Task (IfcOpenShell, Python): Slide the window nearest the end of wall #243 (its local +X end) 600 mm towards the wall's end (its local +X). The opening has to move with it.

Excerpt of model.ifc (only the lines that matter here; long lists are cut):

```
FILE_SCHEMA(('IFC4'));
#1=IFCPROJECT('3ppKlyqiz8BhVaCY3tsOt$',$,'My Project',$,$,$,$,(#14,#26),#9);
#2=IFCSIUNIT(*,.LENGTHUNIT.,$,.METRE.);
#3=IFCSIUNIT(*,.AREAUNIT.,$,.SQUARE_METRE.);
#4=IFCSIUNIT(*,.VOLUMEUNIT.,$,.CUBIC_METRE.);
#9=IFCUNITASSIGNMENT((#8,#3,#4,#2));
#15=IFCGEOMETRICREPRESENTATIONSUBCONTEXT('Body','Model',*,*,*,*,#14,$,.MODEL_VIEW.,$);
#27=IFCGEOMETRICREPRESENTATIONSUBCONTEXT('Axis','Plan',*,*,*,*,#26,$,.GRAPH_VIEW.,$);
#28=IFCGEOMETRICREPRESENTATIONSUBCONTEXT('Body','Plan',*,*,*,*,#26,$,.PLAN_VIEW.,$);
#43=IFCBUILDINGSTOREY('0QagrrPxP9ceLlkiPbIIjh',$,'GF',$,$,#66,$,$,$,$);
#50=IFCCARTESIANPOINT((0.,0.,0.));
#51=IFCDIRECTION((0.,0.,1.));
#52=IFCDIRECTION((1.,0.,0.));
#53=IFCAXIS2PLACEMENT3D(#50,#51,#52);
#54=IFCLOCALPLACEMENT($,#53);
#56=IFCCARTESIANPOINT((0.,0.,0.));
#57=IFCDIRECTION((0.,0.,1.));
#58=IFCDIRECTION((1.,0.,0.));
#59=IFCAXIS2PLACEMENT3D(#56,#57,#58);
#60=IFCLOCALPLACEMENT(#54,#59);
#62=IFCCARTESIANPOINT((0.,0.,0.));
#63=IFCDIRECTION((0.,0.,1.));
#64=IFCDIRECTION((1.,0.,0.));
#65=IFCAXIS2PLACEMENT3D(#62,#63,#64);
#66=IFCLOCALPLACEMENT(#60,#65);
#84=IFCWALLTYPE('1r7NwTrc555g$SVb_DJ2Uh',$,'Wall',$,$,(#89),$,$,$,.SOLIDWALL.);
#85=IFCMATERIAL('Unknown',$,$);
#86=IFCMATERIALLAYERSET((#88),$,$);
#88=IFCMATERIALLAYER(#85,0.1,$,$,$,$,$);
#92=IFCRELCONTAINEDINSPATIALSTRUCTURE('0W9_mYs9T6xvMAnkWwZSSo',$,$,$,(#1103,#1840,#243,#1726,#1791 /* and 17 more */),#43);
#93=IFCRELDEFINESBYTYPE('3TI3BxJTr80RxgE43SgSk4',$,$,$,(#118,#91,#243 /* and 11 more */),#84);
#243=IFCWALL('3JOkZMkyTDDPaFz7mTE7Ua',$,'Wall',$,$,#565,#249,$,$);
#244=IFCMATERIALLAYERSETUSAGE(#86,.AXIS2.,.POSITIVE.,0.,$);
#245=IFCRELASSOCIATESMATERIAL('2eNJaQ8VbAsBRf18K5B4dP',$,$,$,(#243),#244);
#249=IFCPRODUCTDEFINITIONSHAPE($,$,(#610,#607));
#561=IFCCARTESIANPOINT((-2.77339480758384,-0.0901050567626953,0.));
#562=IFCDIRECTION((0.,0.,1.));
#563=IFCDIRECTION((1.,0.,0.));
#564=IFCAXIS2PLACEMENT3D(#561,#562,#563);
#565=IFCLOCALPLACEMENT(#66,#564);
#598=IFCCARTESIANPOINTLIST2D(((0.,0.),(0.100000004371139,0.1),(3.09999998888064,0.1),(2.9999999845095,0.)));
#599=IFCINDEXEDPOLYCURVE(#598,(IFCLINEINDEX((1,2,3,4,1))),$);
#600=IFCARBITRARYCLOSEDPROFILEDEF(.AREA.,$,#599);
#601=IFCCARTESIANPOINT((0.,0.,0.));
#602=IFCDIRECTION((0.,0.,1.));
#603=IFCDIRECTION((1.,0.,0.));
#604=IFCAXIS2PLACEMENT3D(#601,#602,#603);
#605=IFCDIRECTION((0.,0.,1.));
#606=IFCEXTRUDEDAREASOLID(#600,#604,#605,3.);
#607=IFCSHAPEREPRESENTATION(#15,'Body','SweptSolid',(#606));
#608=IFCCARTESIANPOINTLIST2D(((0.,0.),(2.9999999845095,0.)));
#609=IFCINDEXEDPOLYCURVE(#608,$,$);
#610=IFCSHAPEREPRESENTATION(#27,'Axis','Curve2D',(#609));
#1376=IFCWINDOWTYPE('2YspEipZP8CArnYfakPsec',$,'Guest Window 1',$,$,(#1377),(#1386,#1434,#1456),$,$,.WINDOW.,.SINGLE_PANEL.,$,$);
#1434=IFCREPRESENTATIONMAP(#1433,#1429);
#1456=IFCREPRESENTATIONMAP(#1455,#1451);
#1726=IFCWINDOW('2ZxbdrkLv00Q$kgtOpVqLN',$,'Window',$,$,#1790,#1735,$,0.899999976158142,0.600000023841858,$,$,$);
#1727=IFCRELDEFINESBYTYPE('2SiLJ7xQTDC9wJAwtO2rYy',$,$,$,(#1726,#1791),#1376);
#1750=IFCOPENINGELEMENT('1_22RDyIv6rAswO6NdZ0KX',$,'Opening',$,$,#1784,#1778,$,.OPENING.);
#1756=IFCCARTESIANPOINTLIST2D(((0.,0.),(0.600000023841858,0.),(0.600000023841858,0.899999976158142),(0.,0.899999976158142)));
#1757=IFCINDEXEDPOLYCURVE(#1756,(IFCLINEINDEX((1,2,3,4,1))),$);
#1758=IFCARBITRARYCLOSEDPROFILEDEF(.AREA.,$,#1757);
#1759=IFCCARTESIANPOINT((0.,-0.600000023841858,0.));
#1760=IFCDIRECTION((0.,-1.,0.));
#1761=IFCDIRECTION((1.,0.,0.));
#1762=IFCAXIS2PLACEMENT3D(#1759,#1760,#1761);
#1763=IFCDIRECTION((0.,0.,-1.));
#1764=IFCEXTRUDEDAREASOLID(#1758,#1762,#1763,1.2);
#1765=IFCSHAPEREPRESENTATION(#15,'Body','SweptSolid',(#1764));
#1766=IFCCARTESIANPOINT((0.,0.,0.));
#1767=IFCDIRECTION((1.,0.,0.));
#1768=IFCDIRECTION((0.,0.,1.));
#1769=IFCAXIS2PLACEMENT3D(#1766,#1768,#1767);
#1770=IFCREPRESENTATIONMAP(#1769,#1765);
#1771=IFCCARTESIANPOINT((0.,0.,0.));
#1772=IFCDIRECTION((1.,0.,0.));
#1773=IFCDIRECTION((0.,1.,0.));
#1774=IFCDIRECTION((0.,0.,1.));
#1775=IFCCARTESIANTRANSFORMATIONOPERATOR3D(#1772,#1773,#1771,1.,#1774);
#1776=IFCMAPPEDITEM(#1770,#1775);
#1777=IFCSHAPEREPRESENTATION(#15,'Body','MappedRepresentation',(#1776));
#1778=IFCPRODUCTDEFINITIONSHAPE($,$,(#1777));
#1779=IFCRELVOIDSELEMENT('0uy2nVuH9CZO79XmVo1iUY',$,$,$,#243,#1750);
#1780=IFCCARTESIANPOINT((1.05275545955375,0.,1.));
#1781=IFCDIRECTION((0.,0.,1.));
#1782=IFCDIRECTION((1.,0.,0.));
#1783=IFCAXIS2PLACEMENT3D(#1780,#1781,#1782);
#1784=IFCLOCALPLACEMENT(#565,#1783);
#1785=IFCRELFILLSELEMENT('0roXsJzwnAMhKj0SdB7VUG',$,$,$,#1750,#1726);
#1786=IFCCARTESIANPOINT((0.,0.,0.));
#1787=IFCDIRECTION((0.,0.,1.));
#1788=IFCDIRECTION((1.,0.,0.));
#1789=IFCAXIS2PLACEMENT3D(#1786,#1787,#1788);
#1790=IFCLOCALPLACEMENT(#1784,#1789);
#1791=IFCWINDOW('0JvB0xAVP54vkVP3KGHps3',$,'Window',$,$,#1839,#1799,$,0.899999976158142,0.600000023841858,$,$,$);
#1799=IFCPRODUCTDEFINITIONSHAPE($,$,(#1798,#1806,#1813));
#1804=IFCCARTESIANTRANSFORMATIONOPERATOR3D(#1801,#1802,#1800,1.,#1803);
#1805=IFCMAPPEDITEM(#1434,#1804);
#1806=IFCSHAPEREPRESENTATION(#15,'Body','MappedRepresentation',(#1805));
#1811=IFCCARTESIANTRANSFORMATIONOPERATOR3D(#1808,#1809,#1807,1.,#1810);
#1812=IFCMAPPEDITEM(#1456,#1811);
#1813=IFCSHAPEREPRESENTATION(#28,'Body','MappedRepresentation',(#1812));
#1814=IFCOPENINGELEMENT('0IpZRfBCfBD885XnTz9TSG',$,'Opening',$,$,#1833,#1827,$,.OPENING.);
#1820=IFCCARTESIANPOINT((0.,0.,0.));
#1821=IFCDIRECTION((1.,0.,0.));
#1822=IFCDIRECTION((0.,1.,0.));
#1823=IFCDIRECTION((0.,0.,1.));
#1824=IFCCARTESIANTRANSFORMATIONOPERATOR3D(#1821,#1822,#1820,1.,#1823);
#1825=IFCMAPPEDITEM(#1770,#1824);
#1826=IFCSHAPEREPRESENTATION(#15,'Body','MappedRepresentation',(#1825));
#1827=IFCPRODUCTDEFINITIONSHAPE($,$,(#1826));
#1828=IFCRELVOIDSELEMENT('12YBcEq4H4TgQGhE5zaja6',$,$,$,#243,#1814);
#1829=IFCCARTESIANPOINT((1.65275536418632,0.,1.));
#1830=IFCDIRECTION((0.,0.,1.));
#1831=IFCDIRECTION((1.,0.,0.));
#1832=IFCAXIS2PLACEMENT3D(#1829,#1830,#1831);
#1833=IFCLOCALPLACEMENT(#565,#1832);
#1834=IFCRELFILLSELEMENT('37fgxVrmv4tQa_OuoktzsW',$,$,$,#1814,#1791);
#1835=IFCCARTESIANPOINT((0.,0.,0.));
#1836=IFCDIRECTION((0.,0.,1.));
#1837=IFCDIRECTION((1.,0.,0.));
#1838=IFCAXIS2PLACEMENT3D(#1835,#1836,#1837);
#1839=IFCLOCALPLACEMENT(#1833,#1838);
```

```python
import ifcopenshell
import ifcopenshell.api.geometry
import ifcopenshell.util.placement
import ifcopenshell.util.unit

model = ifcopenshell.open("model.ifc")
unit_scale = ifcopenshell.util.unit.calculate_unit_scale(model)

window = model.by_guid("0JvB0xAVP54vkVP3KGHps3")
opening = window.FillsVoids[0].RelatingOpeningElement
wall = opening.VoidsElements[0].RelatingBuildingElement

wall_matrix = ifcopenshell.util.placement.get_local_placement(wall.ObjectPlacement)
shift = wall_matrix[:3, 0] * 0.6 / unit_scale
before = ifcopenshell.util.placement.get_local_placement(window.ObjectPlacement)[:3, 3].copy()

# The window is placed relative to its opening, so it follows when the opening moves.
matrix = ifcopenshell.util.placement.get_local_placement(opening.ObjectPlacement)
matrix[:3, 3] += shift
ifcopenshell.api.geometry.edit_object_placement(
    model, product=opening, matrix=matrix, is_si=False, should_transform_children=True
)

after = ifcopenshell.util.placement.get_local_placement(window.ObjectPlacement)[:3, 3]
print("window moved by", (after - before).round(3) + 0.0)

model.write("model-out.ifc")
```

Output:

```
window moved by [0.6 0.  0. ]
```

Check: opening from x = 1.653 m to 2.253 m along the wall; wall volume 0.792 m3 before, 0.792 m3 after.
